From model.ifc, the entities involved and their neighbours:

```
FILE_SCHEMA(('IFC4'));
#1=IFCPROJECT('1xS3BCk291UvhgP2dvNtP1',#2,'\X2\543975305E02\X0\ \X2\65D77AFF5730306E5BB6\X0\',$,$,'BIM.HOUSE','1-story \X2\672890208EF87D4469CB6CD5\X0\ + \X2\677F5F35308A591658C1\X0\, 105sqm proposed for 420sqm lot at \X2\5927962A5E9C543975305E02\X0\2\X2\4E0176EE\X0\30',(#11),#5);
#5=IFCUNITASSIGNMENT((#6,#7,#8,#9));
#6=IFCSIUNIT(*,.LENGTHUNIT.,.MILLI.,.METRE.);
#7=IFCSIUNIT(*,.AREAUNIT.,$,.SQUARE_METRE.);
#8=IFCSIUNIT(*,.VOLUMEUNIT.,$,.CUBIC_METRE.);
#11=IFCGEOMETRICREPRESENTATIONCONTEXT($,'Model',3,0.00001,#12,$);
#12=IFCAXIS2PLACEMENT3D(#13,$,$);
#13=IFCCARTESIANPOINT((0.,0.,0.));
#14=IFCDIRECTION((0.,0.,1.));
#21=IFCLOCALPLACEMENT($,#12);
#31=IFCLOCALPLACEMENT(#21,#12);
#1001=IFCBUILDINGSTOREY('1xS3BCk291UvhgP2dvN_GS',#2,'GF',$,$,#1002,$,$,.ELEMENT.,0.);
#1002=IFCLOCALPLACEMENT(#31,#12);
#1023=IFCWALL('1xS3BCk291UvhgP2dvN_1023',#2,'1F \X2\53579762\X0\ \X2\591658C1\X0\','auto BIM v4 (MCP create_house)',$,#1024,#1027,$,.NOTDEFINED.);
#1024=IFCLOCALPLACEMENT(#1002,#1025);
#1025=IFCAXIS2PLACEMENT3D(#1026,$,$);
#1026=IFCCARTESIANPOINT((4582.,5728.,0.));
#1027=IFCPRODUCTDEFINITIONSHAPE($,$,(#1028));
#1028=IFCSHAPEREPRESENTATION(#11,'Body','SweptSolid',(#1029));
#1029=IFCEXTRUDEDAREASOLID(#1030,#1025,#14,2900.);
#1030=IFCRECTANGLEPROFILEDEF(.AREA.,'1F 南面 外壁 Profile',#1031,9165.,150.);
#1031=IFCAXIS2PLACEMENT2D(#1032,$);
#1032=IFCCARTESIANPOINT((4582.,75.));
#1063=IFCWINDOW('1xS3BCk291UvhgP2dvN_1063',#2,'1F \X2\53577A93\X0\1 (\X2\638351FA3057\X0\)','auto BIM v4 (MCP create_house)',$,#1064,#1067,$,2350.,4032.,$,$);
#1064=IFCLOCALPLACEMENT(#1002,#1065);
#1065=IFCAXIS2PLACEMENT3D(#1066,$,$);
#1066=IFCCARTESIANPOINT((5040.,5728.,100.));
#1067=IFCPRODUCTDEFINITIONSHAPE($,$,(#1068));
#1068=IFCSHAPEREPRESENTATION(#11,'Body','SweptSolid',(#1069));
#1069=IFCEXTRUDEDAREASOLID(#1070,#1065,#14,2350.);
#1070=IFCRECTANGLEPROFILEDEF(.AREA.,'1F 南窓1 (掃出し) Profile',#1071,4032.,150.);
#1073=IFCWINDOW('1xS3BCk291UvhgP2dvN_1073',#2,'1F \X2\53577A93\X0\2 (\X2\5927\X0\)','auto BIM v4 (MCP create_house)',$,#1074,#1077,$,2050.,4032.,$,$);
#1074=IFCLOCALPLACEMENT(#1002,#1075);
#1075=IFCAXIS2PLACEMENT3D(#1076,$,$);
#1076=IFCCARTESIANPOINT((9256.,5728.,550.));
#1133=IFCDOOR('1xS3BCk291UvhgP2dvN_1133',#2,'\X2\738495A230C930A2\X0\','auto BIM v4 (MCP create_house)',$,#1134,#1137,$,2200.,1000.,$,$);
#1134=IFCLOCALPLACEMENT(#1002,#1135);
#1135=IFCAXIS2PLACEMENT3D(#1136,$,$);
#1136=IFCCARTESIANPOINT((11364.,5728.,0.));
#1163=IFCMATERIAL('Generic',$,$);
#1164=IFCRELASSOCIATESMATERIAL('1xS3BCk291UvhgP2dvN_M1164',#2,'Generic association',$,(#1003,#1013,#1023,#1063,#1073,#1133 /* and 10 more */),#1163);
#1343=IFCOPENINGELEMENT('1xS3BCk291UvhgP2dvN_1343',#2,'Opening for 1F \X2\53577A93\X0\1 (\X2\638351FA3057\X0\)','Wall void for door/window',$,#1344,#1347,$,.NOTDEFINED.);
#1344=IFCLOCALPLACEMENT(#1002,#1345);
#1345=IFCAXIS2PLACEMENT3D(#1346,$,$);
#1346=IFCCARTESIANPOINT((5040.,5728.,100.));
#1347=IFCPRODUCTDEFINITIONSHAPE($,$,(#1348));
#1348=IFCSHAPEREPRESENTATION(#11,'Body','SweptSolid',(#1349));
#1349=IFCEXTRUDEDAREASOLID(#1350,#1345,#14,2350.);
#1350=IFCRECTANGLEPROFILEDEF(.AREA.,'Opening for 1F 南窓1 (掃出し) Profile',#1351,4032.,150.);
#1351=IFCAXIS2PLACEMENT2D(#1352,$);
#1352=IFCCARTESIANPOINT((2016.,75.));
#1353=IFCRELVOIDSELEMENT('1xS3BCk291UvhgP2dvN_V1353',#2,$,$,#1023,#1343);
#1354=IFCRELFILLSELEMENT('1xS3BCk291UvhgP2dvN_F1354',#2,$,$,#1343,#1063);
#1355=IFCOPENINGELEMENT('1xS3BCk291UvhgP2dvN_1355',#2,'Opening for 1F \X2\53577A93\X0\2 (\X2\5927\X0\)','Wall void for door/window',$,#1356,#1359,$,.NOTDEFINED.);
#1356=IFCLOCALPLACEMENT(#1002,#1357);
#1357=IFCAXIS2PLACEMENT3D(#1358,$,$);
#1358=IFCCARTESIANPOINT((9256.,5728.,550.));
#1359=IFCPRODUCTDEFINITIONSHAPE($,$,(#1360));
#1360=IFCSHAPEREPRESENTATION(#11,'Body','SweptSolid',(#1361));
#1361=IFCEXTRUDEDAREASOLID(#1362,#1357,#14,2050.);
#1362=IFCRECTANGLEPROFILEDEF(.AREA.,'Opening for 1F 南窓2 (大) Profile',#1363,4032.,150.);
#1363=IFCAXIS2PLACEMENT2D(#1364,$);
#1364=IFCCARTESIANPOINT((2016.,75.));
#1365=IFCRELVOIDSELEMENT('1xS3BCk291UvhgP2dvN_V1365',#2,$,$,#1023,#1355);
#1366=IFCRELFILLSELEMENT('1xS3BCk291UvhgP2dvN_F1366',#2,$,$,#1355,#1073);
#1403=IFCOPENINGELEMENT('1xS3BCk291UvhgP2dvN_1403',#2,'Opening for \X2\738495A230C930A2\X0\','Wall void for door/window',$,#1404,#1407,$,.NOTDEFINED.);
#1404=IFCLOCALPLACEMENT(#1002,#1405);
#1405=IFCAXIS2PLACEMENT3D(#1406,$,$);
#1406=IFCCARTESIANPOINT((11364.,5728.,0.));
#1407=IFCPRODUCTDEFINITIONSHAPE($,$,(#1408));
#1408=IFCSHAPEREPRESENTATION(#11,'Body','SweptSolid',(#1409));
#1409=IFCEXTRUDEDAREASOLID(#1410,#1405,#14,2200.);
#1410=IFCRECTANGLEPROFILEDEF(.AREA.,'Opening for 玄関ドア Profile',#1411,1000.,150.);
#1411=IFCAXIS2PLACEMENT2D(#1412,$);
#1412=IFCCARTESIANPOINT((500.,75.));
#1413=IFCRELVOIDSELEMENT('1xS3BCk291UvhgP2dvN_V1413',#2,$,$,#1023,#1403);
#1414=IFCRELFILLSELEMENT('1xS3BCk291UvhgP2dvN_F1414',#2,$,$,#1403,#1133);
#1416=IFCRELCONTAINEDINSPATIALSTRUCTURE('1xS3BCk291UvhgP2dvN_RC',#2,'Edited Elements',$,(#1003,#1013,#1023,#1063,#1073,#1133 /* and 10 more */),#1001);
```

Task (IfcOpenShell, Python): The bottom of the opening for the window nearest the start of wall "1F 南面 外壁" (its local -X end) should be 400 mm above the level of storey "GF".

```python
import numpy as np
import ifcopenshell
import ifcopenshell.api.geometry
import ifcopenshell.geom
import ifcopenshell.util.element
import ifcopenshell.util.placement
import ifcopenshell.util.shape
import ifcopenshell.util.unit

model = ifcopenshell.open("model.ifc")
unit_scale = ifcopenshell.util.unit.calculate_unit_scale(model)

window = model.by_guid("1xS3BCk291UvhgP2dvN_1063")
opening = window.FillsVoids[0].RelatingOpeningElement
storey = ifcopenshell.util.element.get_container(window, ifc_class="IfcBuildingStorey")
level = ifcopenshell.util.placement.get_local_placement(storey.ObjectPlacement)[2, 3]

# The opening's origin need not be at the sill, so measure its lowest point.
shape = ifcopenshell.geom.create_shape(ifcopenshell.geom.settings(), opening)
bottom = ifcopenshell.util.shape.get_shape_bottom_elevation(shape, shape.geometry) / unit_scale
dz = level + 400.0 - bottom

shift = np.array([0.0, 0.0, dz])
# The window is not placed relative to its opening, so move both.
for product in (opening, window):
    matrix = ifcopenshell.util.placement.get_local_placement(product.ObjectPlacement)
    matrix[:3, 3] += shift
    ifcopenshell.api.geometry.edit_object_placement(model, product=product, matrix=matrix, is_si=False)

print(f"moved by {dz * unit_scale:+.3f} m")

model.write("model-out.ifc")
```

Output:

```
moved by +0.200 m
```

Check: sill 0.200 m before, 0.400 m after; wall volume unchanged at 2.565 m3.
